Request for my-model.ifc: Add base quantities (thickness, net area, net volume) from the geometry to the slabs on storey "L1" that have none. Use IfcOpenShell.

First a look at what the model holds.

```python
import ifcopenshell
import ifcopenshell.util.element
import ifcopenshell.util.unit

model = ifcopenshell.open("my-model.ifc")
print(model.schema)
for unit_type in ("LENGTHUNIT", "AREAUNIT", "VOLUMEUNIT"):
    print(unit_type, ifcopenshell.util.unit.calculate_unit_scale(model, unit_type))
storey = next(s for s in model.by_type("IfcBuildingStorey") if s.Name == "L1")
slabs = [e for e in ifcopenshell.util.element.get_decomposition(storey) if e.is_a("IfcSlab")]
for e in sorted(slabs, key=lambda e: e.id()):
    print(e.id(), e.is_a(), e.Name, list(ifcopenshell.util.element.get_psets(e, qtos_only=True)), sep=" | ")
```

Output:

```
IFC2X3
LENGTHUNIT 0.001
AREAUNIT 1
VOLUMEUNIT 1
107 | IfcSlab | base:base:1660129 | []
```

```python
import ifcopenshell
import ifcopenshell.api.pset
import ifcopenshell.geom
import ifcopenshell.util.element
import ifcopenshell.util.shape
import ifcopenshell.util.unit

model = ifcopenshell.open("my-model.ifc")
unit_scale = ifcopenshell.util.unit.calculate_unit_scale(model)
area_scale = ifcopenshell.util.unit.calculate_unit_scale(model, "AREAUNIT")
volume_scale = ifcopenshell.util.unit.calculate_unit_scale(model, "VOLUMEUNIT")
settings = ifcopenshell.geom.settings()

storey = next(s for s in model.by_type("IfcBuildingStorey") if s.Name == "L1")
slabs = [e for e in ifcopenshell.util.element.get_decomposition(storey) if e.is_a("IfcSlab")]

for e in sorted(slabs, key=lambda e: e.id()):
    if ifcopenshell.util.element.get_psets(e, qtos_only=True, should_inherit=False):
        continue
    # Geometry comes back in metres, in the element's own axes.
    shape = ifcopenshell.geom.create_shape(settings, e)
    values = {
        "Width": ifcopenshell.util.shape.get_z(shape.geometry) / unit_scale,
        "NetArea": ifcopenshell.util.shape.get_footprint_area(shape.geometry) / area_scale,
        "NetVolume": ifcopenshell.util.shape.get_volume(shape.geometry) / volume_scale,
    }
    qto = ifcopenshell.api.pset.add_qto(model, product=e, name="BaseQuantities")
    ifcopenshell.api.pset.edit_qto(model, qto=qto, properties=values)
    print(e.id(), {k: round(v, 3) for k, v in values.items()})

model.write("my-model_updated.ifc")
```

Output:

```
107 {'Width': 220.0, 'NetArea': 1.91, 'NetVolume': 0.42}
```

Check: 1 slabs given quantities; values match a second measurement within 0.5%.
